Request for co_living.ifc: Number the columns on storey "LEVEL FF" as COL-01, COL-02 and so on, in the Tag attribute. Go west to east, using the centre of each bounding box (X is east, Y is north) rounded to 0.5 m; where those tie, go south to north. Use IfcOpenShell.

First a look at what the model holds.

```python
import ifcopenshell
import ifcopenshell.util.element
import ifcopenshell.util.placement

model = ifcopenshell.open("co_living.ifc")
print(model.schema)
storey = next(s for s in model.by_type("IfcBuildingStorey") if s.Name == "LEVEL FF")
columns = [e for e in ifcopenshell.util.element.get_decomposition(storey) if e.is_a("IfcColumn")]
for e in sorted(columns, key=lambda e: e.id()):
    origin = ifcopenshell.util.placement.get_local_placement(e.ObjectPlacement)[:3, 3]
    print(e.id(), e.Tag, e.Name, origin.round(2) + 0.0, sep=" | ")
```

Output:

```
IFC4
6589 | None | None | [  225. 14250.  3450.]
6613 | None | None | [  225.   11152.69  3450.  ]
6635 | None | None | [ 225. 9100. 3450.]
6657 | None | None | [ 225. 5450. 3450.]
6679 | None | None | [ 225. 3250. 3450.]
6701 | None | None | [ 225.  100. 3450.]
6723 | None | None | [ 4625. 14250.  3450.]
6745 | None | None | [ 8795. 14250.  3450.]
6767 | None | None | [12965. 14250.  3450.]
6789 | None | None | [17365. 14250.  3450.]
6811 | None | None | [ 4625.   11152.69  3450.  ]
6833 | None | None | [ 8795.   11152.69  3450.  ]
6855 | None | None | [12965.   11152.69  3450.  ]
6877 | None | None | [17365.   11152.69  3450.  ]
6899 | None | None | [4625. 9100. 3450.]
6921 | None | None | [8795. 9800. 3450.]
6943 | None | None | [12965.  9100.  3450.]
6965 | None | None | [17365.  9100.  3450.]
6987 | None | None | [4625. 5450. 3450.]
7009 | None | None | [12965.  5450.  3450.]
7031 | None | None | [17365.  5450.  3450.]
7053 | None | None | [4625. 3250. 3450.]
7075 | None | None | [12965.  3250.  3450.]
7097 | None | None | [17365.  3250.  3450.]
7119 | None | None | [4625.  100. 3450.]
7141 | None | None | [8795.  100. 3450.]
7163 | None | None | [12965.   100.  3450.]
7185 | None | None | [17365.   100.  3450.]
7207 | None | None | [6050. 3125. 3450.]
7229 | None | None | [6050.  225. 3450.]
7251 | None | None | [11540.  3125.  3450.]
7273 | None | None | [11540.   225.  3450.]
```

```python
import ifcopenshell
import ifcopenshell.geom
import ifcopenshell.util.element
import ifcopenshell.util.shape

model = ifcopenshell.open("co_living.ifc")
settings = ifcopenshell.geom.settings()
settings.set("use-world-coords", True)


def centre(element):
    shape = ifcopenshell.geom.create_shape(settings, element)
    return ifcopenshell.util.shape.get_bbox_centroid(shape.geometry)


storey = next(s for s in model.by_type("IfcBuildingStorey") if s.Name == "LEVEL FF")
columns = [e for e in ifcopenshell.util.element.get_decomposition(storey) if e.is_a("IfcColumn")]

# Insertion points can sit at a corner or the storey origin, so sort by the geometry (in metres).
centres = {e: centre(e) for e in columns}
columns.sort(key=lambda e: (round(centres[e][0] / 0.5), centres[e][1]))

for i, e in enumerate(columns, start=1):
    number = f"COL-{i:02d}"
    e.Tag = number
    print(e.id(), number)

model.write("co_living_updated.ifc")
```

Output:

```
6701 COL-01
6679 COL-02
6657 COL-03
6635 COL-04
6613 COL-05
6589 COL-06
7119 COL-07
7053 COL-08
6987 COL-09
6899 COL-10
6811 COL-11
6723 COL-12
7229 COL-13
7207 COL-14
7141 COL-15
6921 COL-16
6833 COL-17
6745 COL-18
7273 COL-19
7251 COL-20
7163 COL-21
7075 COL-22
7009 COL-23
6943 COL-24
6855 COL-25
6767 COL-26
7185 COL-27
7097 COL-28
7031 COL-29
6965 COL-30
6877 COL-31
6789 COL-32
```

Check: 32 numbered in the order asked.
